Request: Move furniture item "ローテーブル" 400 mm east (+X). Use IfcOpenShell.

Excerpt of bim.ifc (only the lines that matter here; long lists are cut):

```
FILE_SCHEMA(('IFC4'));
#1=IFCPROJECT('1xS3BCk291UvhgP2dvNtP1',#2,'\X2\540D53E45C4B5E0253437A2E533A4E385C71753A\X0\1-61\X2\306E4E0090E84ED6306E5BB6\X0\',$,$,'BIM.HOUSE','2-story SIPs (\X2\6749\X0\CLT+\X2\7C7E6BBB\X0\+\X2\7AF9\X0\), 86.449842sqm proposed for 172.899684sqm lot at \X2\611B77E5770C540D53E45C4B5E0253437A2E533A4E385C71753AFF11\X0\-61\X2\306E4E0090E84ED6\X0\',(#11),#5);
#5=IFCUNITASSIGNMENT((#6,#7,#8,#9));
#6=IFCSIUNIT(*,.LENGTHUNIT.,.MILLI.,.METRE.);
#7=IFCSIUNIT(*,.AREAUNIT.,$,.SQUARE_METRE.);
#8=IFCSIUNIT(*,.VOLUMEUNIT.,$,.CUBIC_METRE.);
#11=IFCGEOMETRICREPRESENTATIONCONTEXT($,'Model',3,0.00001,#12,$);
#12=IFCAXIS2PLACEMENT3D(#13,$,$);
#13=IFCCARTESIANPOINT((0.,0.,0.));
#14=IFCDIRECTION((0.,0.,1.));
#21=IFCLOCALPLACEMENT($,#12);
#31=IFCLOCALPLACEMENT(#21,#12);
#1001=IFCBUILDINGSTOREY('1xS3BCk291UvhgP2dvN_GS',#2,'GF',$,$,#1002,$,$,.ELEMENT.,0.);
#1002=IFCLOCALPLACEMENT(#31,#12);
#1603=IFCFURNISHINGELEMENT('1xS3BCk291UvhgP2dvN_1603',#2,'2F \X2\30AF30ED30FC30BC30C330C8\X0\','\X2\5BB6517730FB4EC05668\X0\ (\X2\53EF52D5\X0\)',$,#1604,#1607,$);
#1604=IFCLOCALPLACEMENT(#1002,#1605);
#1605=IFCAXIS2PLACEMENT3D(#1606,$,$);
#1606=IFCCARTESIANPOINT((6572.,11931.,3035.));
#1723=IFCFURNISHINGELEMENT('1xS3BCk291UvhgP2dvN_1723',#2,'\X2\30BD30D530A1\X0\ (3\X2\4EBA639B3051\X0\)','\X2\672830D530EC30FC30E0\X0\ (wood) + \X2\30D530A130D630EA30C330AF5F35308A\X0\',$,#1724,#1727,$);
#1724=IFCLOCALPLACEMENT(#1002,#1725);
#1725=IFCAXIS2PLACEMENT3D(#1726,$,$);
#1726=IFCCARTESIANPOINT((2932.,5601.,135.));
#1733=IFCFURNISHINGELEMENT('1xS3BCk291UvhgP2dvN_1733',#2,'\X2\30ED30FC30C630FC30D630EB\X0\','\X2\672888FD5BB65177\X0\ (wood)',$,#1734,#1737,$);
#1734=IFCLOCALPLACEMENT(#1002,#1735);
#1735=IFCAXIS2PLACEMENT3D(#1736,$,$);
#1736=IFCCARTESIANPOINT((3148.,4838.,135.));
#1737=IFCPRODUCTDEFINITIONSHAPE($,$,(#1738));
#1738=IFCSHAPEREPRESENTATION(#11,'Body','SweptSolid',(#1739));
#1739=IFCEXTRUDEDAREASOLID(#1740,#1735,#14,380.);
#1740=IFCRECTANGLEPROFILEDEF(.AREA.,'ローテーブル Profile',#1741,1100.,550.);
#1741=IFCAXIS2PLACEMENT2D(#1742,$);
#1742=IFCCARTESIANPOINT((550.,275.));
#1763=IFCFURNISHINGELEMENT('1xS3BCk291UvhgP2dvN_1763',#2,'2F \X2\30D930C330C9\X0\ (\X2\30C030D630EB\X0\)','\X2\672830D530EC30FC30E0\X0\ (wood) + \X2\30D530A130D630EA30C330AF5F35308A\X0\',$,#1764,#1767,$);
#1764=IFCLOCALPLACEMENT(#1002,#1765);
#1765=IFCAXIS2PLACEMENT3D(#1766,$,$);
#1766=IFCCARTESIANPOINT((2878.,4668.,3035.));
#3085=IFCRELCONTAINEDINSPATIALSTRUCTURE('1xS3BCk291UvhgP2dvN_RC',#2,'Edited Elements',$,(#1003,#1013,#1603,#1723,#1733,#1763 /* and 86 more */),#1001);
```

```python
import ifcopenshell
import ifcopenshell.api.geometry
import ifcopenshell.util.placement

model = ifcopenshell.open("bim.ifc")

item = model.by_guid("1xS3BCk291UvhgP2dvN_1733")
matrix = ifcopenshell.util.placement.get_local_placement(item.ObjectPlacement)
matrix[0, 3] += 400.0
ifcopenshell.api.geometry.edit_object_placement(model, product=item, matrix=matrix, is_si=False)

print(ifcopenshell.util.placement.get_local_placement(item.ObjectPlacement).round(3) + 0.0)

model.write("bim-out.ifc")
```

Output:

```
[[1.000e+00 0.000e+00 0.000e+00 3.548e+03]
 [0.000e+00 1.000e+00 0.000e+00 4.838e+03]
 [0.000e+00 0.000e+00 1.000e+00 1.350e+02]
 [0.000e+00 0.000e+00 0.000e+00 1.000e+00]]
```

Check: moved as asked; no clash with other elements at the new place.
